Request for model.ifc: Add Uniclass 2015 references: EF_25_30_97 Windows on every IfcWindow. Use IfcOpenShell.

First a look at what the model holds.

```python
import ifcopenshell

model = ifcopenshell.open("model.ifc")
print(model.schema)
print("classifications:", [c.Name for c in model.by_type("IfcClassification")])
for ifc_class in ("IfcDoor", "IfcRoof", "IfcStair", "IfcWall", "IfcWindow"):
    print(ifc_class, len(model.by_type(ifc_class)))
```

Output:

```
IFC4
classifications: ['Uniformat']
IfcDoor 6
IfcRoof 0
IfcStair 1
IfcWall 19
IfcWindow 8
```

```python
import ifcopenshell
import ifcopenshell.api.classification

model = ifcopenshell.open("model.ifc")

system = ifcopenshell.api.classification.add_classification(model, classification="Uniclass 2015")

codes = {
    "IfcWindow": ("EF_25_30_97", "Windows"),
}
for ifc_class, (code, name) in codes.items():
    products = model.by_type(ifc_class)
    ifcopenshell.api.classification.add_reference(
        model, products=products, classification=system, identification=code, name=name
    )
    print(code, len(products))

model.write("model-out.ifc")
```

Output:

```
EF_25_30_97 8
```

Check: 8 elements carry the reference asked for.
